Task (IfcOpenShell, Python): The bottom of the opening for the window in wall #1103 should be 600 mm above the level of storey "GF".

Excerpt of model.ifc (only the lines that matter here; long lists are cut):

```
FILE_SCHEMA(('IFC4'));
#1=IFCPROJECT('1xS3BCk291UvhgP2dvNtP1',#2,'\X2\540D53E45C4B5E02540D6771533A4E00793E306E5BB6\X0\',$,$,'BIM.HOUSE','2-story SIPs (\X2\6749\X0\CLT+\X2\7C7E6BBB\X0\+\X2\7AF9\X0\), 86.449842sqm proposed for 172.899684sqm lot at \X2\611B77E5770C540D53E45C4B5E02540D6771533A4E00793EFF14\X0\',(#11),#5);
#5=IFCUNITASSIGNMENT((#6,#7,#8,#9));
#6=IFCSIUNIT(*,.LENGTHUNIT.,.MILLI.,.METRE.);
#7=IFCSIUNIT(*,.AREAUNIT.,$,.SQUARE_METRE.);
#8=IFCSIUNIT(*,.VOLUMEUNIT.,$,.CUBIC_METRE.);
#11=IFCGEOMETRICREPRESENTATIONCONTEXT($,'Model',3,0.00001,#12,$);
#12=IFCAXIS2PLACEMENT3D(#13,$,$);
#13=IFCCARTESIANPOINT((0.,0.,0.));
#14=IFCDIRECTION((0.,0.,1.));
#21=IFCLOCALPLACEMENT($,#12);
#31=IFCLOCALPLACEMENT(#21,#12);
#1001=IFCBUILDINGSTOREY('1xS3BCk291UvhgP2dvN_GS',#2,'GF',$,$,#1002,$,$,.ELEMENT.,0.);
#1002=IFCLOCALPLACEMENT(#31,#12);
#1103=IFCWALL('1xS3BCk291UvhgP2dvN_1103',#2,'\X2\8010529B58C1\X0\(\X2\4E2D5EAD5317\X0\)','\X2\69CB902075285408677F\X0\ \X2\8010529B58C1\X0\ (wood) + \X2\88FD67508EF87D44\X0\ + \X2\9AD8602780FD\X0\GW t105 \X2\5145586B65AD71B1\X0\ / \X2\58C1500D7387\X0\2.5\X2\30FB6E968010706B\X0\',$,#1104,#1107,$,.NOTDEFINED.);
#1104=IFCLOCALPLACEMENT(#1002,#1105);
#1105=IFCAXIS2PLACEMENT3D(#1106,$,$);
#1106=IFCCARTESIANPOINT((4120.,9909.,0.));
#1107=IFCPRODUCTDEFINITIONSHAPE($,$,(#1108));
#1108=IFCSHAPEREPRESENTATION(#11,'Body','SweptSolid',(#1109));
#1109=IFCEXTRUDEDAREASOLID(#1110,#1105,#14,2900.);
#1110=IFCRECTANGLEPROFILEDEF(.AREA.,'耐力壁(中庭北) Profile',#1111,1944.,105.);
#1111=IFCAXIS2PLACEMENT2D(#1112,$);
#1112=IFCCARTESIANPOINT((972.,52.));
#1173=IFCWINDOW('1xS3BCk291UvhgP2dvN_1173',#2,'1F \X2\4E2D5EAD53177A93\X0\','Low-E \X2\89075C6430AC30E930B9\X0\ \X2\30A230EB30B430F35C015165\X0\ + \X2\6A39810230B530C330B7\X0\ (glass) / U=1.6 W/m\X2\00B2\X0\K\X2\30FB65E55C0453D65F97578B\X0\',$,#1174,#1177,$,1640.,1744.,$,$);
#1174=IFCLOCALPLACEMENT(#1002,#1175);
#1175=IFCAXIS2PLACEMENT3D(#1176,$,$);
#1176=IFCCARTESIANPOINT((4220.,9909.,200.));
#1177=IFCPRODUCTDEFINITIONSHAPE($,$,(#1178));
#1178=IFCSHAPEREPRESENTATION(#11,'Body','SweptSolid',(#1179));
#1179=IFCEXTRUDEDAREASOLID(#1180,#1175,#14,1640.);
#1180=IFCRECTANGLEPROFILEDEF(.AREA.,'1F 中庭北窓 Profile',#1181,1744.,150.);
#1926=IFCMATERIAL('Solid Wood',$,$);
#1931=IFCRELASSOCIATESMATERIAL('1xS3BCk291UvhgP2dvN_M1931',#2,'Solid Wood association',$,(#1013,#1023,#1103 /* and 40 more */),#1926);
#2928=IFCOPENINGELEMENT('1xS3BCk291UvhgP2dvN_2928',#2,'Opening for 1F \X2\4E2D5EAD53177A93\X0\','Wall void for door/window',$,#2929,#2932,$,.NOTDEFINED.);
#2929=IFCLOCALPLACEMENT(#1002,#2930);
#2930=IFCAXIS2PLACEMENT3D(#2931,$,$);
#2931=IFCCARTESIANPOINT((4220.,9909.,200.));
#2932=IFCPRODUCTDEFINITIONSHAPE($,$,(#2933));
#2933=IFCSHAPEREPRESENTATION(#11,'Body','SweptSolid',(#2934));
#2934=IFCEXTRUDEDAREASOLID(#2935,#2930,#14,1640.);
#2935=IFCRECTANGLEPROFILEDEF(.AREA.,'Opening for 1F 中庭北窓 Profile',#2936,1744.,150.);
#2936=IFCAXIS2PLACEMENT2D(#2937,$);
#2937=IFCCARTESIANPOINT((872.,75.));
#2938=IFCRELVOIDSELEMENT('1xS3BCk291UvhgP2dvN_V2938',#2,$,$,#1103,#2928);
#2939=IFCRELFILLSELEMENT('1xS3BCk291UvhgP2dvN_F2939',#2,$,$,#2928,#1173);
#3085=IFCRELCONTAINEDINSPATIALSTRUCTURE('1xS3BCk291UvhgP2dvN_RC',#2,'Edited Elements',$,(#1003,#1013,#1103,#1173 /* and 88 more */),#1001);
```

```python
import numpy as np
import ifcopenshell
import ifcopenshell.api.geometry
import ifcopenshell.geom
import ifcopenshell.util.element
import ifcopenshell.util.placement
import ifcopenshell.util.shape
import ifcopenshell.util.unit

model = ifcopenshell.open("model.ifc")
unit_scale = ifcopenshell.util.unit.calculate_unit_scale(model)

window = model.by_id(1173)
opening = window.FillsVoids[0].RelatingOpeningElement
storey = ifcopenshell.util.element.get_container(window, ifc_class="IfcBuildingStorey")
level = ifcopenshell.util.placement.get_local_placement(storey.ObjectPlacement)[2, 3]

# The opening's origin need not be at the sill, so measure its lowest point.
shape = ifcopenshell.geom.create_shape(ifcopenshell.geom.settings(), opening)
bottom = ifcopenshell.util.shape.get_shape_bottom_elevation(shape, shape.geometry) / unit_scale
dz = level + 0.6 / unit_scale - bottom

shift = np.array([0.0, 0.0, dz])
# The window is not placed relative to its opening, so move both.
for product in (opening, window):
    matrix = ifcopenshell.util.placement.get_local_placement(product.ObjectPlacement)
    matrix[:3, 3] += shift
    ifcopenshell.api.geometry.edit_object_placement(model, product=product, matrix=matrix, is_si=False)

print(f"moved by {dz * unit_scale:+.3f} m")

model.write("model_edited.ifc")
```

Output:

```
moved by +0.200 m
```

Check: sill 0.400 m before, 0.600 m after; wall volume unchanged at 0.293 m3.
